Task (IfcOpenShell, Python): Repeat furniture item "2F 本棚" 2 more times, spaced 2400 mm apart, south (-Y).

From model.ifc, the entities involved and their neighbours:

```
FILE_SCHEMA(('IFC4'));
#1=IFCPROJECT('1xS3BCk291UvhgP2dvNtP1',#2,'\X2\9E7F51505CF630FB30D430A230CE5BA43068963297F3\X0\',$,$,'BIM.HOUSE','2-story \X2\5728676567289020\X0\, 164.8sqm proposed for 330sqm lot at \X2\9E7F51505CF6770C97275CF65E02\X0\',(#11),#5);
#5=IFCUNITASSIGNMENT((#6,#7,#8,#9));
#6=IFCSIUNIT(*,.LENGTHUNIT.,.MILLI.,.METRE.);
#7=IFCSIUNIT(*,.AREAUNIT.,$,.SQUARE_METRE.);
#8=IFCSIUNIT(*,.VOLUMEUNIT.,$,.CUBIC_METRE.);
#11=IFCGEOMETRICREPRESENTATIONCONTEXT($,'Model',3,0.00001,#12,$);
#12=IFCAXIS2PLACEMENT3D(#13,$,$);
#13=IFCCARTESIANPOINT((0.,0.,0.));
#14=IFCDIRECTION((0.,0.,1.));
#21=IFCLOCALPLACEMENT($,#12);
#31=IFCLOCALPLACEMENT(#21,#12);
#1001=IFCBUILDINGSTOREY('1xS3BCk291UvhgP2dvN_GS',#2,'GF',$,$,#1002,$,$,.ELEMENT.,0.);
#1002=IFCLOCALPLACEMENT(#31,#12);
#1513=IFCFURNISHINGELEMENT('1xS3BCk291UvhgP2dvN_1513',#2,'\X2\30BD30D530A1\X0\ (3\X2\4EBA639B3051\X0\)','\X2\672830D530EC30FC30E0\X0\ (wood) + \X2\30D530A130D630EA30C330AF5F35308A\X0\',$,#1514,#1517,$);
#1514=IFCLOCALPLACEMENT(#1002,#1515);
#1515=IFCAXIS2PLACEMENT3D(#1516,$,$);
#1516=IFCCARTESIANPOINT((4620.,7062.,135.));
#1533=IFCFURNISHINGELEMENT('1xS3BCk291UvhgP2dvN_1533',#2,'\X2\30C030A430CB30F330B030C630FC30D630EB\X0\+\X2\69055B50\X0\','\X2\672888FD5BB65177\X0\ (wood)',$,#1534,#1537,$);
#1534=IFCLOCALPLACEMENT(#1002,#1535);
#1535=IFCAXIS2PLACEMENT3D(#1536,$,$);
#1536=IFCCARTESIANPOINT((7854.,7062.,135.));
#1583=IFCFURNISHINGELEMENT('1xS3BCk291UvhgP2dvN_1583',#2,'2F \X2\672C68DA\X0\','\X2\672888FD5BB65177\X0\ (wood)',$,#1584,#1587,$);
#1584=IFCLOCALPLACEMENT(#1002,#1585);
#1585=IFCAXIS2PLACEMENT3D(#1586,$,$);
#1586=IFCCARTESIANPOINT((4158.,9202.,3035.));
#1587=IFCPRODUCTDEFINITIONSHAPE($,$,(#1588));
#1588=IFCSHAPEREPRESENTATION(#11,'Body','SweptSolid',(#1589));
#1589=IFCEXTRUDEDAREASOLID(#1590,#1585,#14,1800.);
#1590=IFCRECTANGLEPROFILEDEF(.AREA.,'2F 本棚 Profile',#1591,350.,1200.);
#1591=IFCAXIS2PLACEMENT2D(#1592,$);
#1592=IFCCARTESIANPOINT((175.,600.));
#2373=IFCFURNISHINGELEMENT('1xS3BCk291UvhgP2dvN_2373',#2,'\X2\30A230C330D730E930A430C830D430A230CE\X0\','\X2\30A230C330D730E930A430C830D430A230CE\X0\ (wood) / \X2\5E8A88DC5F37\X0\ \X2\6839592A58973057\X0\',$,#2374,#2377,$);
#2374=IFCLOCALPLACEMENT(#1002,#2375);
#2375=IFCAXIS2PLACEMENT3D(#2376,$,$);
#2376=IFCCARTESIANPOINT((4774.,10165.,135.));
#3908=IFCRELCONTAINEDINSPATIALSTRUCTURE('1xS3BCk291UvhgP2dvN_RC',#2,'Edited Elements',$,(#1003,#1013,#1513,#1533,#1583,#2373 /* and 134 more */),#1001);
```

```python
import numpy as np
import ifcopenshell
import ifcopenshell.api.geometry
import ifcopenshell.api.root
import ifcopenshell.util.element
import ifcopenshell.util.placement
import ifcopenshell.util.unit

model = ifcopenshell.open("model.ifc")
unit_scale = ifcopenshell.util.unit.calculate_unit_scale(model)


def reuse_history(source, copy):
    """copy_class also copies each property set's owner history, people and application; keep the originals."""
    for rel in copy.IsDefinedBy:
        if rel.is_a("IfcRelDefinesByProperties") and (history := rel.RelatingPropertyDefinition.OwnerHistory):
            rel.RelatingPropertyDefinition.OwnerHistory = source.OwnerHistory
            ifcopenshell.util.element.remove_deep2(model, history)


source = model.by_guid("1xS3BCk291UvhgP2dvN_1583")
base = ifcopenshell.util.placement.get_local_placement(source.ObjectPlacement)
step = np.array([0.0, -1.0, 0.0]) * 2.4 / unit_scale

for i in range(1, 3):
    copy = ifcopenshell.api.root.copy_class(model, product=source)
    copy.Representation = ifcopenshell.util.element.copy_deep(
        model, source.Representation, exclude=["IfcGeometricRepresentationContext", "IfcRepresentationMap"]
    )
    reuse_history(source, copy)
    matrix = base.copy()
    matrix[:3, 3] += i * step
    print("added at", matrix[:3, 3].round(3) + 0.0)
    ifcopenshell.api.geometry.edit_object_placement(model, product=copy, matrix=matrix, is_si=False)

model.write("model_edited.ifc")
```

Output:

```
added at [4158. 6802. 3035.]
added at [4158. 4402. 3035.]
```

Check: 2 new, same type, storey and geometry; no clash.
